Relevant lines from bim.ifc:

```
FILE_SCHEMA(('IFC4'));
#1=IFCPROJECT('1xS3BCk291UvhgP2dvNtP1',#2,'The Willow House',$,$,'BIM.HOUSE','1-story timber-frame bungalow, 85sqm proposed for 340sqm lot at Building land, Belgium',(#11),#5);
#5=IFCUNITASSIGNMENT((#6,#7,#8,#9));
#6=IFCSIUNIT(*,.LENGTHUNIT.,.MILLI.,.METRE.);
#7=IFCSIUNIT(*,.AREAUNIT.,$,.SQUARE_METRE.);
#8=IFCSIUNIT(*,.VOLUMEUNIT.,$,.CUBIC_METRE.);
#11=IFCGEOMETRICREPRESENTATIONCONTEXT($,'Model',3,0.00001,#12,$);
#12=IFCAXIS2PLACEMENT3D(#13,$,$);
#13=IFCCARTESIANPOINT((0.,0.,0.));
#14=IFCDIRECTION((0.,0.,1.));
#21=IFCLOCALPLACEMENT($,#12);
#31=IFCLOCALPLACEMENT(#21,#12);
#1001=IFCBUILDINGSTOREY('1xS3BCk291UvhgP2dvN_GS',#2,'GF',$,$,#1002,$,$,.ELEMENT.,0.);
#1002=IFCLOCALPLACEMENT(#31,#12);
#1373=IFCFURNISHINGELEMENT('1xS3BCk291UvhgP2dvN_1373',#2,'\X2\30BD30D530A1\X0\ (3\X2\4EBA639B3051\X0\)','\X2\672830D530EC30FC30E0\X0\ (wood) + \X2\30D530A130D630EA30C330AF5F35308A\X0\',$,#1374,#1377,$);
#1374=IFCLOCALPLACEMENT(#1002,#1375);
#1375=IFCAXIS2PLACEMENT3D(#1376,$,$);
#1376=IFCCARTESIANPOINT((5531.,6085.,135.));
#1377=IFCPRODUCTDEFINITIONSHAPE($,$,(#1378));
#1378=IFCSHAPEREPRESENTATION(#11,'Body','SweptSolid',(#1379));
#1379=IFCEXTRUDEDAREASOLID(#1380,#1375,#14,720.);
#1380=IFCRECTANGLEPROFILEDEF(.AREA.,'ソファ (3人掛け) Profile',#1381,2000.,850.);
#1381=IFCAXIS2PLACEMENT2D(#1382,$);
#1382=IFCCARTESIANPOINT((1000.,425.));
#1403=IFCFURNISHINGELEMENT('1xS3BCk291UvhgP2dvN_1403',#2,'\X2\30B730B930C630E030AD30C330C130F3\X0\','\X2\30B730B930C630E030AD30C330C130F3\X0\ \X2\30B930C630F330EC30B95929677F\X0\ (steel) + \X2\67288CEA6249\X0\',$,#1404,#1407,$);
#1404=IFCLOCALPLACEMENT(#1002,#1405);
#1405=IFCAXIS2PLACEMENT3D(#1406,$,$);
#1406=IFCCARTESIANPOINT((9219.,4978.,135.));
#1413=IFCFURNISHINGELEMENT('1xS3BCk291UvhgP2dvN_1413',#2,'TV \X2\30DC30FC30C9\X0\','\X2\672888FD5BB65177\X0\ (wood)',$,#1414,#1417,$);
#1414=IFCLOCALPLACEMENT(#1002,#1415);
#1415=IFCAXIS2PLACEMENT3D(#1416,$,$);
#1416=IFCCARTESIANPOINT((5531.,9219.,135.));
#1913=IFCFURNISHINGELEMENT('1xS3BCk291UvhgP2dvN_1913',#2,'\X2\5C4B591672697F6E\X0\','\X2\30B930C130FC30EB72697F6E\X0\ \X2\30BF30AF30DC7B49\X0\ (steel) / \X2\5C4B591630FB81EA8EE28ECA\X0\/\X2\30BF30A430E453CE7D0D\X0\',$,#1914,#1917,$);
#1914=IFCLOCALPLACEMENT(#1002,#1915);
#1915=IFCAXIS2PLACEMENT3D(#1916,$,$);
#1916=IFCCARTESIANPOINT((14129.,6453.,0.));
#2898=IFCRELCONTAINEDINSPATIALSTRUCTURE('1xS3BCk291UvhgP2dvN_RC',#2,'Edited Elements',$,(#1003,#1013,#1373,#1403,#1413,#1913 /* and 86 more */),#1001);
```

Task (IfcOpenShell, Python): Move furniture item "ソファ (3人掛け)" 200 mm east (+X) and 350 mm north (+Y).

```python
import ifcopenshell
import ifcopenshell.api.geometry
import ifcopenshell.util.placement
import ifcopenshell.util.unit

model = ifcopenshell.open("bim.ifc")
unit_scale = ifcopenshell.util.unit.calculate_unit_scale(model)

item = model.by_guid("1xS3BCk291UvhgP2dvN_1373")
matrix = ifcopenshell.util.placement.get_local_placement(item.ObjectPlacement)
matrix[0, 3] += 0.2 / unit_scale
matrix[1, 3] += 0.35 / unit_scale
ifcopenshell.api.geometry.edit_object_placement(model, product=item, matrix=matrix, is_si=False)

print(ifcopenshell.util.placement.get_local_placement(item.ObjectPlacement).round(3) + 0.0)

model.write("bim_rev.ifc")
```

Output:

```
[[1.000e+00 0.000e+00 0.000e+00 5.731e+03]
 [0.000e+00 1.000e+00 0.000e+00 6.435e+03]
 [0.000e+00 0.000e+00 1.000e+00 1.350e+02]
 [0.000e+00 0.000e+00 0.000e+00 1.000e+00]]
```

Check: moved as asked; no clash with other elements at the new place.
